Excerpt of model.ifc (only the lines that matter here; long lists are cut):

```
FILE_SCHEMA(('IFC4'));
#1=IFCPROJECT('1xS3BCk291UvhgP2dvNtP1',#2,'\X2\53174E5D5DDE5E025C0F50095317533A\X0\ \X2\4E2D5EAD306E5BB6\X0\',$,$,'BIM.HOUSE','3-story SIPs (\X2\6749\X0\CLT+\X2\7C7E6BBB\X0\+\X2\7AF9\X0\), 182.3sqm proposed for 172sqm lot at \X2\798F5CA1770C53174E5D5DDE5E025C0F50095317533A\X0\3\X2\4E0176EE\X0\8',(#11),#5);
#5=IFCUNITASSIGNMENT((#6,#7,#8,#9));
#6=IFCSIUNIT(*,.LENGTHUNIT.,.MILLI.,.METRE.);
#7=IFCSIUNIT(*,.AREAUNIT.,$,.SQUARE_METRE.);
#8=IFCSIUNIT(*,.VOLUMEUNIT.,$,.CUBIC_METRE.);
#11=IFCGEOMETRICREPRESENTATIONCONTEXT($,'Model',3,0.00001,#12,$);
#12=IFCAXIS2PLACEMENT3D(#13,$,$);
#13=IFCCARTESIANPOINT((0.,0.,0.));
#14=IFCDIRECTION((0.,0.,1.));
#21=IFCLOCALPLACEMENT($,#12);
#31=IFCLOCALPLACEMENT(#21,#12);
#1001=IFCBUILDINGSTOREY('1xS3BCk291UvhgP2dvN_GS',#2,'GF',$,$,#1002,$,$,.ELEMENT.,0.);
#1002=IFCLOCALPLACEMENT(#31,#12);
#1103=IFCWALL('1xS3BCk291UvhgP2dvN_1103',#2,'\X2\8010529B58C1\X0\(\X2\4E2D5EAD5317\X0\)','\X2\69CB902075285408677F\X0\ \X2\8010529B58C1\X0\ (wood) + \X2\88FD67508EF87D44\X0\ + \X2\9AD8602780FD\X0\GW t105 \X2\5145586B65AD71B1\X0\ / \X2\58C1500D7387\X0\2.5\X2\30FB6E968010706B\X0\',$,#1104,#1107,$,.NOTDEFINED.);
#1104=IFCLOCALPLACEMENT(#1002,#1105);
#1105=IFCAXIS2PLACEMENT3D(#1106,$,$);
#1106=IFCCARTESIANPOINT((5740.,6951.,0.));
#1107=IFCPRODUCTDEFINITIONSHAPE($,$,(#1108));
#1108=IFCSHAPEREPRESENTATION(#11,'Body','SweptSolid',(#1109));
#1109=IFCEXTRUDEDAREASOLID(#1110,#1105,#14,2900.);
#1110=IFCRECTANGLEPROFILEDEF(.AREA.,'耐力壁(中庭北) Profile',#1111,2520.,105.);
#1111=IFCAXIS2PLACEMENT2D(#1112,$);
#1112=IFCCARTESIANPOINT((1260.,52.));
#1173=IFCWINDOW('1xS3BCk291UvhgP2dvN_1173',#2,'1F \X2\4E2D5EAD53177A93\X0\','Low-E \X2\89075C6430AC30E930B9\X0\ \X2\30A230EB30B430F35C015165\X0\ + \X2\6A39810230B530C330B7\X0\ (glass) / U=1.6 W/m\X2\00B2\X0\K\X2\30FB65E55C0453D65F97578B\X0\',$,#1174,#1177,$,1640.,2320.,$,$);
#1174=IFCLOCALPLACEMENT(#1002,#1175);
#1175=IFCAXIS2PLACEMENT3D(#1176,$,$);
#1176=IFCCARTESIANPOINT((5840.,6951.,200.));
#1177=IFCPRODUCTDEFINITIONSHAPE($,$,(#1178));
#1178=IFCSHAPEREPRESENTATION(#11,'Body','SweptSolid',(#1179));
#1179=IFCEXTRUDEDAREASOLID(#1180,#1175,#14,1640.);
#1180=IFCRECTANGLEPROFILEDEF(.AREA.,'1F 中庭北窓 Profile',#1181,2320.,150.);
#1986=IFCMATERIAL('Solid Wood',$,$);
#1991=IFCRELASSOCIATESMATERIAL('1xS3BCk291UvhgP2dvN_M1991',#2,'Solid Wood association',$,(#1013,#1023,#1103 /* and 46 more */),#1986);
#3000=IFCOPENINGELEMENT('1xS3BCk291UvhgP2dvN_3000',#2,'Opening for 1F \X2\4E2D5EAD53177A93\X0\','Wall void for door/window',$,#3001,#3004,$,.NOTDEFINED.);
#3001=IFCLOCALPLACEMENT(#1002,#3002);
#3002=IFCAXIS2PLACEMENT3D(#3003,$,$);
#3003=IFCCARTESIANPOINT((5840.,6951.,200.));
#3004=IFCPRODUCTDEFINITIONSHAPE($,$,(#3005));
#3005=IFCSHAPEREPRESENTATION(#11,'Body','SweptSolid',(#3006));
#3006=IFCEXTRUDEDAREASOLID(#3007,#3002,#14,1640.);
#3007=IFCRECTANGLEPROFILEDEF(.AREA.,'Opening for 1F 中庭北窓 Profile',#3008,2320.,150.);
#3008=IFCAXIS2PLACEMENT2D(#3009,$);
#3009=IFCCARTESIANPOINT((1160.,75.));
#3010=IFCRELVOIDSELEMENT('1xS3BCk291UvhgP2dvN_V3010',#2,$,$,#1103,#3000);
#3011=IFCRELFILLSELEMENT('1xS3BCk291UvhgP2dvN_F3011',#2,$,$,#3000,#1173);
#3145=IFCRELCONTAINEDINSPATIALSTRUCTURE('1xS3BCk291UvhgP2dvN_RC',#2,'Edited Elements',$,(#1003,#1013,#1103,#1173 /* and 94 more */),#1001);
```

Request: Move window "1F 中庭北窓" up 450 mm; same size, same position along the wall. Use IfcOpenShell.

```python
import numpy as np
import ifcopenshell
import ifcopenshell.api.geometry
import ifcopenshell.util.placement
import ifcopenshell.util.unit

model = ifcopenshell.open("model.ifc")
unit_scale = ifcopenshell.util.unit.calculate_unit_scale(model)

window = model.by_id(1173)
opening = window.FillsVoids[0].RelatingOpeningElement
dz = 450.0

shift = np.array([0.0, 0.0, dz])
# The window is not placed relative to its opening, so move both.
for product in (opening, window):
    matrix = ifcopenshell.util.placement.get_local_placement(product.ObjectPlacement)
    matrix[:3, 3] += shift
    ifcopenshell.api.geometry.edit_object_placement(model, product=product, matrix=matrix, is_si=False)

print(f"moved by {dz * unit_scale:+.3f} m")

model.write("model_rev.ifc")
```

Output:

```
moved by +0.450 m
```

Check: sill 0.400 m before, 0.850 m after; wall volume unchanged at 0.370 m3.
